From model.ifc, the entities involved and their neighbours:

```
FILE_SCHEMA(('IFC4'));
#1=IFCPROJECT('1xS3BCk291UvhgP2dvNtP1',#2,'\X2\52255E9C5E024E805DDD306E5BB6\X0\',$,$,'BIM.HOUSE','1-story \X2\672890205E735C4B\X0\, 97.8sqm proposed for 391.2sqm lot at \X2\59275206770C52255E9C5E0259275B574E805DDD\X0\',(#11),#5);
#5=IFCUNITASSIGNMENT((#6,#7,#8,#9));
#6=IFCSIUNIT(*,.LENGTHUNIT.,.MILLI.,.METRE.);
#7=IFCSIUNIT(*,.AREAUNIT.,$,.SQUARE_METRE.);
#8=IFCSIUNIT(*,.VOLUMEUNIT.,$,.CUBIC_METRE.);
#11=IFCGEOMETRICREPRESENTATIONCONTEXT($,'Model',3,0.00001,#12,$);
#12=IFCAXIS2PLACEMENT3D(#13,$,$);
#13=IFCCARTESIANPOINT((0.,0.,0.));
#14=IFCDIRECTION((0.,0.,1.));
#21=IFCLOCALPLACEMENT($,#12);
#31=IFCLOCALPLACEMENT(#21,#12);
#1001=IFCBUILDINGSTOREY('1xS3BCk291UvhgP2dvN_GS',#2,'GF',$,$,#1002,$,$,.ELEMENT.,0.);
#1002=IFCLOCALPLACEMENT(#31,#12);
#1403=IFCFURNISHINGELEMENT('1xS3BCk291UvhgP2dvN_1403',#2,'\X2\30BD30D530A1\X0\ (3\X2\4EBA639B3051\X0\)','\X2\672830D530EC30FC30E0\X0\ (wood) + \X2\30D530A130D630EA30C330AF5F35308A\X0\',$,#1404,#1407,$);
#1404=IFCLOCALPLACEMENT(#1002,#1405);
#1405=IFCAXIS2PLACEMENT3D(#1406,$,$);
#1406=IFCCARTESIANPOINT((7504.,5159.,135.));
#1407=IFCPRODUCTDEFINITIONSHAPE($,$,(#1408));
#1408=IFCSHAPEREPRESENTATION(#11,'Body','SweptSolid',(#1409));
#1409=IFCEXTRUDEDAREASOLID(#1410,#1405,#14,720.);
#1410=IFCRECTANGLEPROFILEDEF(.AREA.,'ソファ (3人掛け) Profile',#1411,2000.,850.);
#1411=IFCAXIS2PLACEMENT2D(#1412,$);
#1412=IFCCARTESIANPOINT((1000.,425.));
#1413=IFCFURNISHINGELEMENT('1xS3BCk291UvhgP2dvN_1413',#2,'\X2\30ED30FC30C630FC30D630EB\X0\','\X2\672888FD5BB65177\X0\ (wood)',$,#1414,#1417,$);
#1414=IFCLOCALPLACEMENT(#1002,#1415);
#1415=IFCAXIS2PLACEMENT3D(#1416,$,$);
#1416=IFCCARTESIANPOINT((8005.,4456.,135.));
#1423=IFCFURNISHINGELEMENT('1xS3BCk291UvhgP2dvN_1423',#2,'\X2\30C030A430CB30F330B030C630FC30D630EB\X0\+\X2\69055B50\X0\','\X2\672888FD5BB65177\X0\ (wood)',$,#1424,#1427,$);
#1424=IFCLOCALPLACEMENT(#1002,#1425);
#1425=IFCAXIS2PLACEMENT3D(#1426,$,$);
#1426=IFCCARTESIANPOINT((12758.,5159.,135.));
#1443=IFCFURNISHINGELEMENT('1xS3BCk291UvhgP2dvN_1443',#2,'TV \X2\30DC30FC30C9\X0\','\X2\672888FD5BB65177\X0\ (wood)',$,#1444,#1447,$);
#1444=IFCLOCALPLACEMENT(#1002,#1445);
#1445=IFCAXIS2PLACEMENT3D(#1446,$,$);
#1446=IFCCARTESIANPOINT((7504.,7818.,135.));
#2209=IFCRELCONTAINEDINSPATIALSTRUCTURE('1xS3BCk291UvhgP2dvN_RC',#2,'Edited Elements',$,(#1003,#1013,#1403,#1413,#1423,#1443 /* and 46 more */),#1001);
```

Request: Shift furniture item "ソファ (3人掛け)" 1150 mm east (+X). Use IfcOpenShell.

```python
import ifcopenshell
import ifcopenshell.api.geometry
import ifcopenshell.util.placement

model = ifcopenshell.open("model.ifc")

item = model.by_guid("1xS3BCk291UvhgP2dvN_1403")
matrix = ifcopenshell.util.placement.get_local_placement(item.ObjectPlacement)
matrix[0, 3] += 1150.0
ifcopenshell.api.geometry.edit_object_placement(model, product=item, matrix=matrix, is_si=False)

print(ifcopenshell.util.placement.get_local_placement(item.ObjectPlacement).round(3) + 0.0)

model.write("model-out.ifc")
```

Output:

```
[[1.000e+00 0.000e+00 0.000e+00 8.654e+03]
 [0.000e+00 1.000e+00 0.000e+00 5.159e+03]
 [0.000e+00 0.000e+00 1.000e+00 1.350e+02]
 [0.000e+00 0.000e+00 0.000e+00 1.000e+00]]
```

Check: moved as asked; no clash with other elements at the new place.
